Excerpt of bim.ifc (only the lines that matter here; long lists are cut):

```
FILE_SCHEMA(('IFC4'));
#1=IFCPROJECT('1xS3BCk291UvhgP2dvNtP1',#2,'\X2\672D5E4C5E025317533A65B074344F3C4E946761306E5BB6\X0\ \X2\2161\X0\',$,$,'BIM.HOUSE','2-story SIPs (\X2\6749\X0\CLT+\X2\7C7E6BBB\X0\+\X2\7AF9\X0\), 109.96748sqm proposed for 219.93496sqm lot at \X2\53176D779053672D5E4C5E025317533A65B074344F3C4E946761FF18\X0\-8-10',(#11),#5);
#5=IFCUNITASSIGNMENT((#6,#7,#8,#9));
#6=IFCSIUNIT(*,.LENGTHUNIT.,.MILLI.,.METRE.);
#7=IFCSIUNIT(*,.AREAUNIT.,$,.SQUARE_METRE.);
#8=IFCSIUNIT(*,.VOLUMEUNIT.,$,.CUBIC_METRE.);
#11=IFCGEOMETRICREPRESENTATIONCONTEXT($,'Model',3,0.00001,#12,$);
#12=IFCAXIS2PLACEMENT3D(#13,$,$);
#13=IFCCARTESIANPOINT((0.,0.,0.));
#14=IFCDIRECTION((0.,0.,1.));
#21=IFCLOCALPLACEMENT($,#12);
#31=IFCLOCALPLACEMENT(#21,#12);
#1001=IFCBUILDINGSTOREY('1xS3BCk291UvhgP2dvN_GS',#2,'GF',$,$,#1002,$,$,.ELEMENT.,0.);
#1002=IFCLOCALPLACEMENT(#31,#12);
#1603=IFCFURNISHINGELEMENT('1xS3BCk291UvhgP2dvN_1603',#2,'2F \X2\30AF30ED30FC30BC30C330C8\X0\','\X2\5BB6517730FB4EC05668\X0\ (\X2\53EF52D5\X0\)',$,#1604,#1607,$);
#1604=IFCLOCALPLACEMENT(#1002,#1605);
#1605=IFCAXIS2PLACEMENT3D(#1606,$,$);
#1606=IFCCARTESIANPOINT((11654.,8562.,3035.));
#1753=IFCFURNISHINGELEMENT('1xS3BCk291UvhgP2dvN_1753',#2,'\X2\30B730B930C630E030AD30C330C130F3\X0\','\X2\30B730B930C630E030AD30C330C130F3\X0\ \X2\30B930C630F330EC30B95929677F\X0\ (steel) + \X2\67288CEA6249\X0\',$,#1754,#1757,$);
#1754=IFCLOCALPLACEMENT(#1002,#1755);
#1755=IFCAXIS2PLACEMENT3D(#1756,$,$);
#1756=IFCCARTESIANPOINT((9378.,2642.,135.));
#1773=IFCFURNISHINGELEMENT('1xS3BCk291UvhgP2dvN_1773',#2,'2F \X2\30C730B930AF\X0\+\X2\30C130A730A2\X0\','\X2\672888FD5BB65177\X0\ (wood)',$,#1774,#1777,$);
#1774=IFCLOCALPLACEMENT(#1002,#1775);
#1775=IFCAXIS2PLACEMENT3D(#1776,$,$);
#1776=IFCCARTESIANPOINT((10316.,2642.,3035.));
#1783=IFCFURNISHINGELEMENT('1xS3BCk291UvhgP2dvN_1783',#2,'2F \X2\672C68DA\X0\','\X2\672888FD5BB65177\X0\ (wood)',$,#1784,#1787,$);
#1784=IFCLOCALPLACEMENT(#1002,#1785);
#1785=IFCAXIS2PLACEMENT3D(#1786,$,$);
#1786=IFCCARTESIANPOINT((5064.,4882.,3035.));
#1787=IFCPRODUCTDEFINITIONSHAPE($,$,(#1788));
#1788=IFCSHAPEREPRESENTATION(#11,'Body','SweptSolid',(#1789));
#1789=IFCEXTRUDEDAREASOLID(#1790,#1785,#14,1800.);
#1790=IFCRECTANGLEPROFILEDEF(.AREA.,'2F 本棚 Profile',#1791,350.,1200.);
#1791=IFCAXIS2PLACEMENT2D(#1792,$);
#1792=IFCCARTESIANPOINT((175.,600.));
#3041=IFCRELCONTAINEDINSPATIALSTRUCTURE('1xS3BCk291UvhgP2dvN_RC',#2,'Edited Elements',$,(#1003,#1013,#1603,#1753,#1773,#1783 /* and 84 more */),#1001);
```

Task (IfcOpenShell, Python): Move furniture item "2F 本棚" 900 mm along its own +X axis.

```python
import ifcopenshell
import ifcopenshell.api.geometry
import ifcopenshell.util.placement

model = ifcopenshell.open("bim.ifc")

item = model.by_id(1783)
matrix = ifcopenshell.util.placement.get_local_placement(item.ObjectPlacement)
matrix[:3, 3] += matrix[:3, 0] * 900.0
ifcopenshell.api.geometry.edit_object_placement(model, product=item, matrix=matrix, is_si=False)

print(ifcopenshell.util.placement.get_local_placement(item.ObjectPlacement).round(3) + 0.0)

model.write("bim_rev.ifc")
```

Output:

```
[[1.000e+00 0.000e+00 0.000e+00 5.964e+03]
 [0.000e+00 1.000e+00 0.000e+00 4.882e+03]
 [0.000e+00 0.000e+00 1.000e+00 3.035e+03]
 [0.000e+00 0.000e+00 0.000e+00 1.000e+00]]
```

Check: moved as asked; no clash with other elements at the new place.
